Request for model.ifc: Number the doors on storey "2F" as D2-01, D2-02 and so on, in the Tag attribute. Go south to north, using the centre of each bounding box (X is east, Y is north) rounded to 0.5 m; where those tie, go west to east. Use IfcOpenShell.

First a look at what the model holds.

```python
import ifcopenshell
import ifcopenshell.util.element
import ifcopenshell.util.placement

model = ifcopenshell.open("model.ifc")
print(model.schema)
storey = next(s for s in model.by_type("IfcBuildingStorey") if s.Name == "2F")
doors = [e for e in ifcopenshell.util.element.get_decomposition(storey) if e.is_a("IfcDoor")]
for e in sorted(doors, key=lambda e: e.id()):
    origin = ifcopenshell.util.placement.get_local_placement(e.ObjectPlacement)[:3, 3]
    print(e.id(), e.Tag, e.Name, origin.round(2) + 0.0, sep=" | ")
```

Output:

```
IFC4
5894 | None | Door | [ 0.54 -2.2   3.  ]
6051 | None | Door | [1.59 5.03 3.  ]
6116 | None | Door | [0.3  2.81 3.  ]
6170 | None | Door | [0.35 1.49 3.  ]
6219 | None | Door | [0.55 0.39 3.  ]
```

```python
import ifcopenshell
import ifcopenshell.geom
import ifcopenshell.util.element
import ifcopenshell.util.shape

model = ifcopenshell.open("model.ifc")
settings = ifcopenshell.geom.settings()
settings.set("use-world-coords", True)


def centre(element):
    shape = ifcopenshell.geom.create_shape(settings, element)
    return ifcopenshell.util.shape.get_bbox_centroid(shape.geometry)


storey = next(s for s in model.by_type("IfcBuildingStorey") if s.Name == "2F")
doors = [e for e in ifcopenshell.util.element.get_decomposition(storey) if e.is_a("IfcDoor")]

# Insertion points can sit at a corner or the storey origin, so sort by the geometry (in metres).
centres = {e: centre(e) for e in doors}
doors.sort(key=lambda e: (round(centres[e][1] / 0.5), centres[e][0]))

for i, e in enumerate(doors, start=1):
    number = f"D2-{i:02d}"
    e.Tag = number
    print(e.id(), number)

model.write("model_edited.ifc")
```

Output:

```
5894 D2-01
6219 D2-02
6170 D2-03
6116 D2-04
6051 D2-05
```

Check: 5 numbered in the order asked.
